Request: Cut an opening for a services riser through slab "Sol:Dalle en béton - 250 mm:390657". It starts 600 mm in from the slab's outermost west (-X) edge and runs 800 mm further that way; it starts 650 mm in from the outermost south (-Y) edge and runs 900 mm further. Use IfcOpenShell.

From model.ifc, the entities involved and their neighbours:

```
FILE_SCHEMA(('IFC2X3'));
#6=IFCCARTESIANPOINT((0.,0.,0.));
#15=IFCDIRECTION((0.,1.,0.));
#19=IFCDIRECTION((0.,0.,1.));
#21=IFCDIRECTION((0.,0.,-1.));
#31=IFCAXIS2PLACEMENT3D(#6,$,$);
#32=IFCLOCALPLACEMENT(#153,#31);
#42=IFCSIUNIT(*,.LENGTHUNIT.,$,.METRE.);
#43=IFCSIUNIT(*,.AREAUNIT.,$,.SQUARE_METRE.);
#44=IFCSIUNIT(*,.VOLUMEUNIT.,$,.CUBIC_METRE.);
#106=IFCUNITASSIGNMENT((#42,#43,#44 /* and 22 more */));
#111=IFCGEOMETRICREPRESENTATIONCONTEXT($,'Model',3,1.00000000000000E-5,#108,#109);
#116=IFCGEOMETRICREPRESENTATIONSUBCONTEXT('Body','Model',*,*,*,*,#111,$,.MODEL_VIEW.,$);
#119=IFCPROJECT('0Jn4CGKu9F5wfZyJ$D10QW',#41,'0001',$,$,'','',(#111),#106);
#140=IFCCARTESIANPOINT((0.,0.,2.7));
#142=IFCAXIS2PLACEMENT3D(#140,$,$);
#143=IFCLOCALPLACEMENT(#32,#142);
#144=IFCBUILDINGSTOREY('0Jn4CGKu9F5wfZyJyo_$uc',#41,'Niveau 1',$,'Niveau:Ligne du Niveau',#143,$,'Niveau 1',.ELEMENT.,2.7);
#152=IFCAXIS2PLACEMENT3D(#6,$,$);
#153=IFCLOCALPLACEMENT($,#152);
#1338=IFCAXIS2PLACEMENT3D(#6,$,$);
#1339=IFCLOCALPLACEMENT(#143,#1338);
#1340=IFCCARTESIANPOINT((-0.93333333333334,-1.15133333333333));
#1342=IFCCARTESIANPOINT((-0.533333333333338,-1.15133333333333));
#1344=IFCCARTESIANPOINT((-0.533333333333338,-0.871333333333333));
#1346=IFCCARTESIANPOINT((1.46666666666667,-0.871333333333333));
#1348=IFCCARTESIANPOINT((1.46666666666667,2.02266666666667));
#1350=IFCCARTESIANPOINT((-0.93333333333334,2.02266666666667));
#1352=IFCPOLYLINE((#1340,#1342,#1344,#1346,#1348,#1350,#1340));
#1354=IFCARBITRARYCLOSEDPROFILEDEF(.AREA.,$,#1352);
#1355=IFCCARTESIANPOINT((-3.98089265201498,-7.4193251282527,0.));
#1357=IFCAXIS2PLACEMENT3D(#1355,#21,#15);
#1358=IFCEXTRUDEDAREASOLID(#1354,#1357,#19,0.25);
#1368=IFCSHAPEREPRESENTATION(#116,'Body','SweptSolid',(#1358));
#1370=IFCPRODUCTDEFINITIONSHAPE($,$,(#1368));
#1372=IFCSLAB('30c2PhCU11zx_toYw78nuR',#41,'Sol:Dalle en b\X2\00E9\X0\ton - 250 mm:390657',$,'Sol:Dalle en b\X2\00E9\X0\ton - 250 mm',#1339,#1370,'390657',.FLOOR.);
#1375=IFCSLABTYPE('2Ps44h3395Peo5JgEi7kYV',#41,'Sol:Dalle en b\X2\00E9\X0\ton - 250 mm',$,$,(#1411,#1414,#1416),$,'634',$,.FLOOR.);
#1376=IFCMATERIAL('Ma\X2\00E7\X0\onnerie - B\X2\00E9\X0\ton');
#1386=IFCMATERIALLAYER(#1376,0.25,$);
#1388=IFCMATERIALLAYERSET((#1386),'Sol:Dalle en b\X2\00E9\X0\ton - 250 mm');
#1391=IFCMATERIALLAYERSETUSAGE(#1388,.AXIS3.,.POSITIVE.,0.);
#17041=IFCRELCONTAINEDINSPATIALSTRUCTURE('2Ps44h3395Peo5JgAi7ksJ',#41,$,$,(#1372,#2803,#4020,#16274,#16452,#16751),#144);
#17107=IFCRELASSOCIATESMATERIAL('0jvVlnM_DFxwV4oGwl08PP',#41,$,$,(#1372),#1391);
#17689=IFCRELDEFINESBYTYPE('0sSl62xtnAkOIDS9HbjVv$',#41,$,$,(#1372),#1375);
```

```python
import numpy as np
import ifcopenshell
import ifcopenshell.api.feature
import ifcopenshell.api.geometry
import ifcopenshell.api.root
import ifcopenshell.geom
import ifcopenshell.util.placement
import ifcopenshell.util.representation
import ifcopenshell.util.shape
import ifcopenshell.util.unit

model = ifcopenshell.open("model.ifc")
unit_scale = ifcopenshell.util.unit.calculate_unit_scale(model)
settings = ifcopenshell.geom.settings()


def volume(element):
    """Net volume in cubic metres, openings subtracted."""
    shape = ifcopenshell.geom.create_shape(settings, element)
    return ifcopenshell.util.shape.get_volume(shape.geometry)


slab = model.by_guid("30c2PhCU11zx_toYw78nuR")
before = volume(slab)

# Extent in the slab's own axes, in metres. The edges named are its -X and -Y sides.
slab_shape = ifcopenshell.geom.create_shape(settings, slab)
vertices = ifcopenshell.util.shape.get_vertices(slab_shape.geometry)
x_min, y_min, bottom = vertices.min(axis=0)
top = vertices[:, 2].max()

opening = ifcopenshell.api.root.create_entity(model, ifc_class="IfcOpeningElement", name="Services riser opening")
context = ifcopenshell.util.representation.get_context(model, "Model", "Body", "MODEL_VIEW")
width, depth = 0.8, 0.9
outline = [(0.0, 0.0), (width, 0.0), (width, depth), (0.0, depth), (0.0, 0.0)]
# Overshoot both faces by 50 mm so the cut is clean.
shape = ifcopenshell.api.geometry.add_slab_representation(
    model, context=context, depth=top - bottom + 0.1, polyline=outline
)
ifcopenshell.api.geometry.assign_representation(model, product=opening, representation=shape)

matrix = ifcopenshell.util.placement.get_local_placement(slab.ObjectPlacement)
matrix[:, 3] = matrix @ np.append(np.array([x_min + 0.6, y_min + 0.65, bottom - 0.05]) / unit_scale, 1.0)
ifcopenshell.api.geometry.edit_object_placement(model, product=opening, matrix=matrix, is_si=False)
ifcopenshell.api.feature.add_feature(model, feature=opening, element=slab)

after = volume(slab)

print(f"slab volume {before:.3f} -> {after:.3f} m3")

model.write("model-out.ifc")
```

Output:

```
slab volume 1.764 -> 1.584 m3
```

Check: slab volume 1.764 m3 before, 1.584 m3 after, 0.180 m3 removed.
